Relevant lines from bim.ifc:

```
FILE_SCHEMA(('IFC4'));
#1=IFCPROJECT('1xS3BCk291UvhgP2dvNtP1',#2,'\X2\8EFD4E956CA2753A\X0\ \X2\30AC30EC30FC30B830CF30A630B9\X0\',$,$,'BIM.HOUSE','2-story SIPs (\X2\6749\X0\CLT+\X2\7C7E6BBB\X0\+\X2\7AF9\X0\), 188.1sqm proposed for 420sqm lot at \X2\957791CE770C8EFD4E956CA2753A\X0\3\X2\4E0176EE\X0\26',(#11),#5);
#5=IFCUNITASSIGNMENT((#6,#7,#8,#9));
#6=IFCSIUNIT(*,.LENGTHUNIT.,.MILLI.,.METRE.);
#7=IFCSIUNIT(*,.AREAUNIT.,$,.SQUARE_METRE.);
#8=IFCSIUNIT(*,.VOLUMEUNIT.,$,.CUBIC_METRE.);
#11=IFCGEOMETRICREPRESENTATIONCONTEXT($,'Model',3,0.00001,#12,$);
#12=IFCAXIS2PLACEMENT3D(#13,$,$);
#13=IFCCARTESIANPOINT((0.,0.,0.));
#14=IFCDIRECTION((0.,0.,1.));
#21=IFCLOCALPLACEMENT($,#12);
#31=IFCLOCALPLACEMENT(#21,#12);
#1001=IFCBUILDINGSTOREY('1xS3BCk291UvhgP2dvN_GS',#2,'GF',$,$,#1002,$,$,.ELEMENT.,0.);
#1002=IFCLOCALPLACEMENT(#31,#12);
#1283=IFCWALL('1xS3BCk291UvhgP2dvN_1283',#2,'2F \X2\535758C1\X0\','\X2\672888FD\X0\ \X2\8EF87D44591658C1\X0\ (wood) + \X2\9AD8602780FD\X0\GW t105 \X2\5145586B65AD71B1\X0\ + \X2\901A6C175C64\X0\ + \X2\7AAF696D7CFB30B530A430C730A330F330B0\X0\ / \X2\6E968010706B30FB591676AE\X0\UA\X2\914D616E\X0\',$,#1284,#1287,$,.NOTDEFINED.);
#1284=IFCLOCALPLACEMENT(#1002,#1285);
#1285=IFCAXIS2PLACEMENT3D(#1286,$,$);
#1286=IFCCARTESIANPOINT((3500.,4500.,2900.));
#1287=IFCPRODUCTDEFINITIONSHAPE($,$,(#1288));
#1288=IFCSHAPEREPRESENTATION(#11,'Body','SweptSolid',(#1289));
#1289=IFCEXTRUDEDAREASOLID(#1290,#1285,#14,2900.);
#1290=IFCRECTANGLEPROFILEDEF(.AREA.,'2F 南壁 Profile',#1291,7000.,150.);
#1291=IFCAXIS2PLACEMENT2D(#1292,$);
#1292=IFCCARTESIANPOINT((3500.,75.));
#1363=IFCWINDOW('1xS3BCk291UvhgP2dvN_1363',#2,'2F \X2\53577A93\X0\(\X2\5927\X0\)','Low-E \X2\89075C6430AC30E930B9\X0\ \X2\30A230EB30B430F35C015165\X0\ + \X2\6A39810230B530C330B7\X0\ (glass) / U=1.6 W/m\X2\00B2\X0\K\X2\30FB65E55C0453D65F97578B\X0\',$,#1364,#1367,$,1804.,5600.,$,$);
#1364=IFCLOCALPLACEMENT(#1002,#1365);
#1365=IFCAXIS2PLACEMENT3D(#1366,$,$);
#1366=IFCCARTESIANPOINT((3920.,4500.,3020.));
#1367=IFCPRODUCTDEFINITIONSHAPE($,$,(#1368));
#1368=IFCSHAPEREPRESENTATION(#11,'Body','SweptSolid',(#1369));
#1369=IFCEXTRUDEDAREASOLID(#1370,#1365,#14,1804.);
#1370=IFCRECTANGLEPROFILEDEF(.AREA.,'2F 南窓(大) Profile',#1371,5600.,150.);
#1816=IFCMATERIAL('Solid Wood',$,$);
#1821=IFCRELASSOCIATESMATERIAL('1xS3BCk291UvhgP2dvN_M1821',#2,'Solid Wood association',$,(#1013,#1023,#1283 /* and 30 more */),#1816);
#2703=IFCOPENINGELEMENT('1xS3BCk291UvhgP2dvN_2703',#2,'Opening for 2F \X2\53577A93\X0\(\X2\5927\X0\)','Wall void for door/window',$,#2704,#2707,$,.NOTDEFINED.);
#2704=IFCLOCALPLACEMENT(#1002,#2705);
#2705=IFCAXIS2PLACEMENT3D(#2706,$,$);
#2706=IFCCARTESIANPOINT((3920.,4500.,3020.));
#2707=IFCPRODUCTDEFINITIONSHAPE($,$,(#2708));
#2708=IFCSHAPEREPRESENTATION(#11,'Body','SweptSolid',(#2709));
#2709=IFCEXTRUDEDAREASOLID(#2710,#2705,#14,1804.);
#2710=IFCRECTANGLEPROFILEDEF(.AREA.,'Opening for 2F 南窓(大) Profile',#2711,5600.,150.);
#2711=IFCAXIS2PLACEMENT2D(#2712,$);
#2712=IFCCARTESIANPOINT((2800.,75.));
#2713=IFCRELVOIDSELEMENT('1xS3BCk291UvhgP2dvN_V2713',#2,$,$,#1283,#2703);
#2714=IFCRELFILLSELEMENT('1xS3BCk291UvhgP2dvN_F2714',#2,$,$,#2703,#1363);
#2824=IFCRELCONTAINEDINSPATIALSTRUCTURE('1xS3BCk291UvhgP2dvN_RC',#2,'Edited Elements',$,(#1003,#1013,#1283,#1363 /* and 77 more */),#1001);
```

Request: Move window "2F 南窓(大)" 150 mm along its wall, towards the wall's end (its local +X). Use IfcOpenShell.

```python
import ifcopenshell
import ifcopenshell.api.geometry
import ifcopenshell.util.placement
import ifcopenshell.util.unit

model = ifcopenshell.open("bim.ifc")
unit_scale = ifcopenshell.util.unit.calculate_unit_scale(model)

window = model.by_guid("1xS3BCk291UvhgP2dvN_1363")
opening = window.FillsVoids[0].RelatingOpeningElement
wall = opening.VoidsElements[0].RelatingBuildingElement

wall_matrix = ifcopenshell.util.placement.get_local_placement(wall.ObjectPlacement)
shift = wall_matrix[:3, 0] * 0.15 / unit_scale
before = ifcopenshell.util.placement.get_local_placement(window.ObjectPlacement)[:3, 3].copy()

# The window is not placed relative to its opening, so move both.
for product in (opening, window):
    matrix = ifcopenshell.util.placement.get_local_placement(product.ObjectPlacement)
    matrix[:3, 3] += shift
    ifcopenshell.api.geometry.edit_object_placement(model, product=product, matrix=matrix, is_si=False)

after = ifcopenshell.util.placement.get_local_placement(window.ObjectPlacement)[:3, 3]
print("window moved by", (after - before).round(3) + 0.0)

model.write("bim-out.ifc")
```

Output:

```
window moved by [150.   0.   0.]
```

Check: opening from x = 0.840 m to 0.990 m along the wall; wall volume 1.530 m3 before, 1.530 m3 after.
